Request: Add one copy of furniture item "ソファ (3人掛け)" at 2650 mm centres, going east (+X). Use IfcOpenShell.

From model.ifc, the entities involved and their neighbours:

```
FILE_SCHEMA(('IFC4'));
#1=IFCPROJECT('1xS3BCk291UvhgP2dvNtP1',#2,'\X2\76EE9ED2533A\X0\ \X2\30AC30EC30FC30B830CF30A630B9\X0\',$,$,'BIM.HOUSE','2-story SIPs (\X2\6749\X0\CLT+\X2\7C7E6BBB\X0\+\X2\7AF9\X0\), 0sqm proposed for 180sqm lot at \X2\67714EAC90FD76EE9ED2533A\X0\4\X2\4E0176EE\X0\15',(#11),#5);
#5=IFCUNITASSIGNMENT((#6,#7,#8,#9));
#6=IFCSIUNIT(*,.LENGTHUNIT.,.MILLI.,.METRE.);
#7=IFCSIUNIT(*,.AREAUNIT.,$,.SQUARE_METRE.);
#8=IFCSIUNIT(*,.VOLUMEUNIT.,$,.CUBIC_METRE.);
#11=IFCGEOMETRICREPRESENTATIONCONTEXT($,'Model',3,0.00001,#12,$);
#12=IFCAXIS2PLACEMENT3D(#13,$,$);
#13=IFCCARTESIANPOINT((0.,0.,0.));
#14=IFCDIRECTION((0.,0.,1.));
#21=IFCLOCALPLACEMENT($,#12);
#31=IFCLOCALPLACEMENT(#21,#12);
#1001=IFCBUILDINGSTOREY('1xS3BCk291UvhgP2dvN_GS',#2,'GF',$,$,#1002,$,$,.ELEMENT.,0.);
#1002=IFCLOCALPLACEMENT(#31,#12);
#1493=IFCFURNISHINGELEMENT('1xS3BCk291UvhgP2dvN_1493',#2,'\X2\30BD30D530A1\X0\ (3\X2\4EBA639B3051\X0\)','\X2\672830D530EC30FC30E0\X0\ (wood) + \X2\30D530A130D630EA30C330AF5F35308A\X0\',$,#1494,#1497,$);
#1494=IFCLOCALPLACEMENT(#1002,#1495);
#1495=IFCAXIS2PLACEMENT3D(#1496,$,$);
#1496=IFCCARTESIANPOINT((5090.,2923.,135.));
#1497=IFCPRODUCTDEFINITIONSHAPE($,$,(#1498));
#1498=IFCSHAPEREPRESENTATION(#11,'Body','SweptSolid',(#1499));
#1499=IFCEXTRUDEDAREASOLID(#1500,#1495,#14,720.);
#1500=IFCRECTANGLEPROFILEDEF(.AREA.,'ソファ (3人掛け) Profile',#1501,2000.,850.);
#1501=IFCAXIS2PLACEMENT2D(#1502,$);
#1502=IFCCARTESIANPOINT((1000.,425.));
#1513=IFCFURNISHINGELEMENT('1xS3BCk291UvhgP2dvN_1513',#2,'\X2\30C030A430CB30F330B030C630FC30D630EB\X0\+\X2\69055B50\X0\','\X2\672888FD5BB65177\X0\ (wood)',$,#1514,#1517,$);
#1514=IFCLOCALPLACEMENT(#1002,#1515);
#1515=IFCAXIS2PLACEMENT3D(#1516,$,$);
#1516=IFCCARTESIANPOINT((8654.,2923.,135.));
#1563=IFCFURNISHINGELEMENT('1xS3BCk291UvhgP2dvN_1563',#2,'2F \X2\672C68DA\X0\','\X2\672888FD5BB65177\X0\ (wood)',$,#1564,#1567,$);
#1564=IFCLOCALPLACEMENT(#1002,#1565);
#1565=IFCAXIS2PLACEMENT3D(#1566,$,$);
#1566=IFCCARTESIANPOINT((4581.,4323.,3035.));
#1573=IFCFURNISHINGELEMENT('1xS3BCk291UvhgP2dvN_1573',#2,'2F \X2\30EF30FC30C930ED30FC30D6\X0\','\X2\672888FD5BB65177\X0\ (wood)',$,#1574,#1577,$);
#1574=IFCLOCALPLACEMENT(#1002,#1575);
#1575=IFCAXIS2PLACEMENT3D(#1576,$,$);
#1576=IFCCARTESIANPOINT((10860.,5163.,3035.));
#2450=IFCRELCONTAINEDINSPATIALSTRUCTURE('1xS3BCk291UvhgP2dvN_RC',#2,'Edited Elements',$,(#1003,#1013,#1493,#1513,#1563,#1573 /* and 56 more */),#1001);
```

```python
import numpy as np
import ifcopenshell
import ifcopenshell.api.geometry
import ifcopenshell.api.root
import ifcopenshell.util.element
import ifcopenshell.util.placement
import ifcopenshell.util.unit

model = ifcopenshell.open("model.ifc")
unit_scale = ifcopenshell.util.unit.calculate_unit_scale(model)


def reuse_history(source, copy):
    """copy_class also copies each property set's owner history, people and application; keep the originals."""
    for rel in copy.IsDefinedBy:
        if rel.is_a("IfcRelDefinesByProperties") and (history := rel.RelatingPropertyDefinition.OwnerHistory):
            rel.RelatingPropertyDefinition.OwnerHistory = source.OwnerHistory
            ifcopenshell.util.element.remove_deep2(model, history)


source = model.by_guid("1xS3BCk291UvhgP2dvN_1493")
base = ifcopenshell.util.placement.get_local_placement(source.ObjectPlacement)
step = np.array([1.0, 0.0, 0.0]) * 2.65 / unit_scale

for i in range(1, 2):
    copy = ifcopenshell.api.root.copy_class(model, product=source)
    copy.Representation = ifcopenshell.util.element.copy_deep(
        model, source.Representation, exclude=["IfcGeometricRepresentationContext", "IfcRepresentationMap"]
    )
    reuse_history(source, copy)
    matrix = base.copy()
    matrix[:3, 3] += i * step
    print("added at", matrix[:3, 3].round(3) + 0.0)
    ifcopenshell.api.geometry.edit_object_placement(model, product=copy, matrix=matrix, is_si=False)

model.write("model-out.ifc")
```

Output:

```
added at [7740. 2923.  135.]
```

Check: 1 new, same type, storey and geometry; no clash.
